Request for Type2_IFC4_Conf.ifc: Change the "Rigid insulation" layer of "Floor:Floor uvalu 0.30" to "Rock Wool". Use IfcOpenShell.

First a look at what the model holds.

```python
import ifcopenshell
import ifcopenshell.util.element

model = ifcopenshell.open("Type2_IFC4_Conf.ifc")
print(model.schema)
for layer_set in model.by_type("IfcMaterialLayerSet"):
    if layer_set.LayerSetName == "Floor:Floor uvalu 0.30":
        for layer in layer_set.MaterialLayers:
            print(layer.id(), layer.Material and layer.Material.Name, layer.LayerThickness, sep=" | ")
        print(len(ifcopenshell.util.element.get_elements_by_material(model, layer_set)), "elements and types use it")
print(sorted(m.Name for m in model.by_type("IfcMaterial") if m.Name)[:60])
```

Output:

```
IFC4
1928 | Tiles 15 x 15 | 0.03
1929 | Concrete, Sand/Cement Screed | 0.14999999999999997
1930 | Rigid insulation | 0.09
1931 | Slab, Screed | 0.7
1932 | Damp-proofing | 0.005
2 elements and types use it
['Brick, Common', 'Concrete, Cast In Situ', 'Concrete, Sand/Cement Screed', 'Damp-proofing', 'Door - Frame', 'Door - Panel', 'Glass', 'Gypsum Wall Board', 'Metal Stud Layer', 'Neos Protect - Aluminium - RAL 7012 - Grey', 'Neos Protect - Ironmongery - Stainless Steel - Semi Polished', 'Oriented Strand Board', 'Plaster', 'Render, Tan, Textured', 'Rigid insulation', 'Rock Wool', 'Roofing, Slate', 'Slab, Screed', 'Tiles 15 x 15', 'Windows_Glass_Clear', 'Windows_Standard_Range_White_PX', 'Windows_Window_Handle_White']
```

```python
import ifcopenshell
import ifcopenshell.api.material

model = ifcopenshell.open("Type2_IFC4_Conf.ifc")

layer_set = next(s for s in model.by_type("IfcMaterialLayerSet") if s.LayerSetName == "Floor:Floor uvalu 0.30")
layer = next(l for l in layer_set.MaterialLayers if l.Material and l.Material.Name == "Rigid insulation")
material = next(m for m in model.by_type("IfcMaterial") if m.Name == "Rock Wool")

# Point this one layer at the other material; renaming the old one would change it everywhere.
ifcopenshell.api.material.edit_layer(model, layer=layer, attributes={"Name": material.Name}, material=material)

print([l.Material.Name if l.Material else None for l in layer_set.MaterialLayers])

model.write("Type2_IFC4_Conf-out.ifc")
```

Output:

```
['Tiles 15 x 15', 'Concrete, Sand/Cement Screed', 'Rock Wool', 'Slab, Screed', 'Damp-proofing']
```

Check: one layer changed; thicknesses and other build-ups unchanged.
